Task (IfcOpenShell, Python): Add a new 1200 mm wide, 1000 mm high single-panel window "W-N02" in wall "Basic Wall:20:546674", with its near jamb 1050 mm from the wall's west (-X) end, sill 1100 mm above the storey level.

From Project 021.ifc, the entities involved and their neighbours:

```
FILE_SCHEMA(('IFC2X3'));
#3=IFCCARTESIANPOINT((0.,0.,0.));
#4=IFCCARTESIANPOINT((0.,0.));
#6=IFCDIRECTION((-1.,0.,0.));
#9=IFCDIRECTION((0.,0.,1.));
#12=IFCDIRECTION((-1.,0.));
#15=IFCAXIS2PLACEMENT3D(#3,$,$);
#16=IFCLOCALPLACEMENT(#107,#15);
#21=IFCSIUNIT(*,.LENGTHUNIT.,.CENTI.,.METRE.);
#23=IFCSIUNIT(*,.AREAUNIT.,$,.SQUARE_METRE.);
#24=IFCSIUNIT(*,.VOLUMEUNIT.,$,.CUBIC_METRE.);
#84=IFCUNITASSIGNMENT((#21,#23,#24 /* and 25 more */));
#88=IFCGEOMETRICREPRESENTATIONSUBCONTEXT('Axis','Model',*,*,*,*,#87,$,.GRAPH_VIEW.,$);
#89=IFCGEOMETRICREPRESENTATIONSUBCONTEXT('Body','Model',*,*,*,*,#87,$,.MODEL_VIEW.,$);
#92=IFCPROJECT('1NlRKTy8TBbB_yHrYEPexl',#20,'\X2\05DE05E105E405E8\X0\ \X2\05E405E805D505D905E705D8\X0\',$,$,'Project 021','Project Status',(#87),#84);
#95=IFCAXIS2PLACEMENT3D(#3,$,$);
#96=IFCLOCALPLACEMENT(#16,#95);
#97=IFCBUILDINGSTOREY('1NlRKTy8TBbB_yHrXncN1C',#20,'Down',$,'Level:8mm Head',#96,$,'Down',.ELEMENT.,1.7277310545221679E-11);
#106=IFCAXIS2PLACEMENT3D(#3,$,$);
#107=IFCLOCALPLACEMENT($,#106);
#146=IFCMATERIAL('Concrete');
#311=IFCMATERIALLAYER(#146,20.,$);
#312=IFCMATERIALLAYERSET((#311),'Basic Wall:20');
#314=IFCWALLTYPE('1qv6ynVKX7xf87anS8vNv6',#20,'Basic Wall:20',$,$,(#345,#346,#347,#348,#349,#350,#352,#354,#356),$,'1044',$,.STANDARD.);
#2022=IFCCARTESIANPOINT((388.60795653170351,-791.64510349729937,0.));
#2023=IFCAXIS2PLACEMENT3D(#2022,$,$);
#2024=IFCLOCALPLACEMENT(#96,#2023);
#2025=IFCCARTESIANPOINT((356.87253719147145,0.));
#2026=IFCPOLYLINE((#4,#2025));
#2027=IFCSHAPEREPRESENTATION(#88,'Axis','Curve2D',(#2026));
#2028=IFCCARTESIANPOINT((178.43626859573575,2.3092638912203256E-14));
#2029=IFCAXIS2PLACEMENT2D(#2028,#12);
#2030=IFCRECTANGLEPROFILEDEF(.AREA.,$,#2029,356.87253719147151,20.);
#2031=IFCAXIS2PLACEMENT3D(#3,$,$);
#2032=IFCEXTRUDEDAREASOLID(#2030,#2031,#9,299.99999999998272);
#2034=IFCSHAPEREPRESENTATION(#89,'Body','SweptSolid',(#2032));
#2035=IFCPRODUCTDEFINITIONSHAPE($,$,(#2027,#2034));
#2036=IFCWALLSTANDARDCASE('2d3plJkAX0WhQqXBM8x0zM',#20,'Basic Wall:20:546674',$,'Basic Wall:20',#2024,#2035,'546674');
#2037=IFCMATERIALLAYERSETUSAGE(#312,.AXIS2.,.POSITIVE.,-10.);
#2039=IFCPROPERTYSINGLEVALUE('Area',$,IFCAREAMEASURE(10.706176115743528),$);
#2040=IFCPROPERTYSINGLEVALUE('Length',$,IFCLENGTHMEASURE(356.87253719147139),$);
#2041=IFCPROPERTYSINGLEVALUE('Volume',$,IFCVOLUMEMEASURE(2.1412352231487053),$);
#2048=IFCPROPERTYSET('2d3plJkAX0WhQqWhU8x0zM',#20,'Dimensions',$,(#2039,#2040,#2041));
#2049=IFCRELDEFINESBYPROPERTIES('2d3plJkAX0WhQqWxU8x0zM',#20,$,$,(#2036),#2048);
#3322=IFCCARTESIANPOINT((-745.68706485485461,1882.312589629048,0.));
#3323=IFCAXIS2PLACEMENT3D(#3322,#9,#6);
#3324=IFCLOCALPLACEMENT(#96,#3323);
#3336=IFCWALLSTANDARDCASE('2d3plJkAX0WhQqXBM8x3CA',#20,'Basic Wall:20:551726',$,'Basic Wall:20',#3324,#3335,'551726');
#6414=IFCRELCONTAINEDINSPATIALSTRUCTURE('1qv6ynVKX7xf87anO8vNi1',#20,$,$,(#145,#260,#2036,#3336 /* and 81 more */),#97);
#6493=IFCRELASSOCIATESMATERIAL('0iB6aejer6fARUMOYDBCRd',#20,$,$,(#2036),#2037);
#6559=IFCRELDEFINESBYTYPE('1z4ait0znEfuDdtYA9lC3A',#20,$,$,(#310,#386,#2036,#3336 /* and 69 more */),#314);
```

```python
import numpy as np
import ifcopenshell
import ifcopenshell.api.feature
import ifcopenshell.api.geometry
import ifcopenshell.api.pset
import ifcopenshell.api.root
import ifcopenshell.api.spatial
import ifcopenshell.api.type
import ifcopenshell.geom
import ifcopenshell.util.element
import ifcopenshell.util.placement
import ifcopenshell.util.representation
import ifcopenshell.util.shape
import ifcopenshell.util.unit

model = ifcopenshell.open("Project 021.ifc")
unit_scale = ifcopenshell.util.unit.calculate_unit_scale(model)
area_scale = ifcopenshell.util.unit.calculate_unit_scale(model, "AREAUNIT")
volume_scale = ifcopenshell.util.unit.calculate_unit_scale(model, "VOLUMEUNIT")
settings = ifcopenshell.geom.settings()


def volume(element):
    """Net volume in cubic metres, openings subtracted."""
    shape = ifcopenshell.geom.create_shape(settings, element)
    return ifcopenshell.util.shape.get_volume(shape.geometry)


wall = model.by_id(2036)
storey = ifcopenshell.util.element.get_container(wall, ifc_class="IfcBuildingStorey")
context = ifcopenshell.util.representation.get_context(model, "Model", "Body", "MODEL_VIEW")
before = volume(wall)

width, height, from_end, sill = 1.2, 1, 1.05, 1.1  # metres

# The wall runs along its own X axis, and the end named is its -X end.
wall_shape = ifcopenshell.geom.create_shape(settings, wall)
x, y, z = ifcopenshell.util.shape.get_vertices(wall_shape.geometry).T
start = x.min() + from_end
face, thickness = float(y.min()), float(y.max() - y.min())
wall_matrix = ifcopenshell.util.placement.get_local_placement(wall.ObjectPlacement)
level = ifcopenshell.util.placement.get_local_placement(storey.ObjectPlacement)[2, 3]


def in_wall(x, y):
    """Placement at x, y metres in the wall's axes, at sill height."""
    matrix = wall_matrix.copy()
    matrix[:, 3] = wall_matrix @ np.array([x / unit_scale, y / unit_scale, 0.0, 1.0])
    matrix[2, 3] = level + sill / unit_scale
    return matrix


# Opening: a box that overshoots both wall faces by 50 mm.
opening = ifcopenshell.api.root.create_entity(model, ifc_class="IfcOpeningElement")
box = ifcopenshell.api.geometry.add_wall_representation(
    model, context=context, length=width, height=height, thickness=thickness + 0.1
)
ifcopenshell.api.geometry.assign_representation(model, product=opening, representation=box)
ifcopenshell.api.geometry.edit_object_placement(model, product=opening, matrix=in_wall(start, face - 0.05), is_si=False)
ifcopenshell.api.feature.add_feature(model, feature=opening, element=wall)

window = ifcopenshell.api.root.create_entity(model, ifc_class="IfcWindow", name="W-N02")
window.OverallWidth, window.OverallHeight = width / unit_scale, height / unit_scale
body = ifcopenshell.api.geometry.add_window_representation(
    model,
    context=context,
    overall_width=window.OverallWidth,
    overall_height=window.OverallHeight,
    partition_type="SINGLE_PANEL",
)
ifcopenshell.api.geometry.assign_representation(model, product=window, representation=body)
ifcopenshell.api.spatial.assign_container(model, products=[window], relating_structure=storey)
fills = ifcopenshell.api.feature.add_filling(model, opening=opening, element=window)
fills.OwnerHistory = window.OwnerHistory  # required in IFC2X3

# IFC2X3 keeps the operation on the window style.
style = ifcopenshell.api.root.create_entity(model, ifc_class="IfcWindowStyle", name="W-N02")
style.OperationType, style.ConstructionType = "SINGLE_PANEL", "NOTDEFINED"
style.ParameterTakesPrecedence = style.Sizeable = False
ifcopenshell.api.type.assign_type(model, related_objects=[window], relating_type=style)

# Centre the window in the wall's thickness.
ifcopenshell.api.geometry.edit_object_placement(model, product=window, matrix=in_wall(start, face), is_si=False)
window_shape = ifcopenshell.geom.create_shape(settings, window)
depth = ifcopenshell.util.shape.get_vertices(window_shape.geometry)[:, 1]
offset = face + thickness / 2 - (depth.min() + depth.max()) / 2
ifcopenshell.api.geometry.edit_object_placement(model, product=window, matrix=in_wall(start, offset), is_si=False)

after = volume(wall)

# Update the wall's stored quantities.
pset = model.by_id(ifcopenshell.util.element.get_pset(wall, "Dimensions", should_inherit=False)["id"])
ifcopenshell.api.pset.edit_pset(model, pset=pset, properties={
    "Area": model.create_entity("IfcAreaMeasure", after / thickness / area_scale),
    "Volume": model.create_entity("IfcVolumeMeasure", after / volume_scale),
})

print(f"wall volume {before:.3f} -> {after:.3f} m3")

model.write("Project 021-out.ifc")
```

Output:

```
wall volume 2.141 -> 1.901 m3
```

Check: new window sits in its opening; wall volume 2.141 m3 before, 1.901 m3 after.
